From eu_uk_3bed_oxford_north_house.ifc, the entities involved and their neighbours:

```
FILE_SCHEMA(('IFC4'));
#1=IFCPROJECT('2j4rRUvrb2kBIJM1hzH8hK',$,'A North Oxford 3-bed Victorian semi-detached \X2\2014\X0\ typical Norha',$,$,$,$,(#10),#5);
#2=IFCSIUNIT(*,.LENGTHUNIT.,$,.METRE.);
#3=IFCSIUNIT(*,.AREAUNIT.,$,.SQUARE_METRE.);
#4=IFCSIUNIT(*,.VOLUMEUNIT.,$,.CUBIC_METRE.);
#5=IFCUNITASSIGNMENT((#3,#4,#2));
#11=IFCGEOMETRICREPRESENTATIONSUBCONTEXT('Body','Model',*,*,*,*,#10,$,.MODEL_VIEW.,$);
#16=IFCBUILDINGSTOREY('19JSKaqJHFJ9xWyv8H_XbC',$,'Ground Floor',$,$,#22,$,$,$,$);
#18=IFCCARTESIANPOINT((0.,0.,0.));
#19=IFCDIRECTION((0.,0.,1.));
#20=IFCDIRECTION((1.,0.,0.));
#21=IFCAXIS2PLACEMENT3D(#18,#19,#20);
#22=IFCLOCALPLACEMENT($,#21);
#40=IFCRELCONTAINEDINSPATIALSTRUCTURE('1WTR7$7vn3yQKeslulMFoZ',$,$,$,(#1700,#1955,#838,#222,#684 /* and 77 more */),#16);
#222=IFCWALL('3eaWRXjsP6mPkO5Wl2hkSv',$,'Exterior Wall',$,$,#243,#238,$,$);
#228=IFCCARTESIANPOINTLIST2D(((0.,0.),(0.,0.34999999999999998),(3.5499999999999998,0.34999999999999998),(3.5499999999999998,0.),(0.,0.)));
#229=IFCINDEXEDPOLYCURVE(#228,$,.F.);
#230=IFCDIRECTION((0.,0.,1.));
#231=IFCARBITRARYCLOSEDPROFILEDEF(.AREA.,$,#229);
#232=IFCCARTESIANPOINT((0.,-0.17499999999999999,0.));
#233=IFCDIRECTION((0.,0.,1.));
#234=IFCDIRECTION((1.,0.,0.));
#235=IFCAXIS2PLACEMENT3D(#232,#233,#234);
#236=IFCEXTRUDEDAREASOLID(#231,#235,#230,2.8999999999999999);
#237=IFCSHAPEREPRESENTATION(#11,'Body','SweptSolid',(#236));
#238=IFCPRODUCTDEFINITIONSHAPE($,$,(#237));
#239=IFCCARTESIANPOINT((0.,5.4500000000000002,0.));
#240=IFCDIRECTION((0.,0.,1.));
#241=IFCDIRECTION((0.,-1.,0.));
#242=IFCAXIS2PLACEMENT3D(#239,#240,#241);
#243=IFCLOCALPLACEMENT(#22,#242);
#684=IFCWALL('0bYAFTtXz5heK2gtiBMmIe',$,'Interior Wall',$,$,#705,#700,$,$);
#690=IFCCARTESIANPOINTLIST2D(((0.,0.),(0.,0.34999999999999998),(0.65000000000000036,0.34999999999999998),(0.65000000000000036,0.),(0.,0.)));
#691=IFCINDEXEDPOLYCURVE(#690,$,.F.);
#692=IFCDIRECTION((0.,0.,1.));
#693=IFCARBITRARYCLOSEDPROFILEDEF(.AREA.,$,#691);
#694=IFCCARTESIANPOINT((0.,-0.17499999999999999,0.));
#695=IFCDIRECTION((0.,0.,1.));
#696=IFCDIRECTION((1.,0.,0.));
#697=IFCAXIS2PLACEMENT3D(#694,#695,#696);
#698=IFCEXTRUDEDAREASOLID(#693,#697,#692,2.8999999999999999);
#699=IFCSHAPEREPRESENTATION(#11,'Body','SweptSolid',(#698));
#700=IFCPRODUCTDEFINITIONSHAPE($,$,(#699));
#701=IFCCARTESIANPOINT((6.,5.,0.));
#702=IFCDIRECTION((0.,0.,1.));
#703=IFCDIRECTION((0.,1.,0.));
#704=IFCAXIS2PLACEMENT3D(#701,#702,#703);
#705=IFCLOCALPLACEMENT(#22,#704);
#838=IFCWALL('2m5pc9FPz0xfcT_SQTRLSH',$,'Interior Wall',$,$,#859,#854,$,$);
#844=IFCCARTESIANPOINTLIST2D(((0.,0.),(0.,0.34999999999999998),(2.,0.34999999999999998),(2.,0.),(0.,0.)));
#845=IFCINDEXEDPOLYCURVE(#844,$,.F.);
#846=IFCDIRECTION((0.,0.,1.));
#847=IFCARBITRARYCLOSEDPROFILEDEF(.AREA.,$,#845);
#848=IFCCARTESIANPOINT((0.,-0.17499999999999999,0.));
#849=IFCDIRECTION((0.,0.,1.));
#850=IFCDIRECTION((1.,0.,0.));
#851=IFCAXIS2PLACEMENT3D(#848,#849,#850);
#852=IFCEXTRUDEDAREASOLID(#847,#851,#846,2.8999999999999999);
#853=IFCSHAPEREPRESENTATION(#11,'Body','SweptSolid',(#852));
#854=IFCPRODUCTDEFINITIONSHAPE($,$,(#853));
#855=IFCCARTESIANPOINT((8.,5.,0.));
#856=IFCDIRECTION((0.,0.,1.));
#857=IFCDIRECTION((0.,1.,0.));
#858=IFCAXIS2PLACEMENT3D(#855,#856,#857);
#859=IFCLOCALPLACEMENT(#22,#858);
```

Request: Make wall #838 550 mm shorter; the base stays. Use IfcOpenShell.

```python
import ifcopenshell
import ifcopenshell.geom
import ifcopenshell.util.representation
import ifcopenshell.util.shape
import ifcopenshell.util.unit

model = ifcopenshell.open("eu_uk_3bed_oxford_north_house.ifc")
unit_scale = ifcopenshell.util.unit.calculate_unit_scale(model)
settings = ifcopenshell.geom.settings()


def volume(element):
    """Net volume in cubic metres, openings subtracted."""
    shape = ifcopenshell.geom.create_shape(settings, element)
    return ifcopenshell.util.shape.get_volume(shape.geometry)


wall = model.by_guid("2m5pc9FPz0xfcT_SQTRLSH")
before = volume(wall)

body = ifcopenshell.util.representation.get_representation(wall, "Model", "Body")
solid = body.Items[0]
old_height = solid.Depth
solid.Depth -= 0.55 / unit_scale
after = volume(wall)

print(f"height {old_height:g} -> {solid.Depth:g}, volume {before:.3f} -> {after:.3f} m3")

model.write("eu_uk_3bed_oxford_north_house_edited.ifc")
```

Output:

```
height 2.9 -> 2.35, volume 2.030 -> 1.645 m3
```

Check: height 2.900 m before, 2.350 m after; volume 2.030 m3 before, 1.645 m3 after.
